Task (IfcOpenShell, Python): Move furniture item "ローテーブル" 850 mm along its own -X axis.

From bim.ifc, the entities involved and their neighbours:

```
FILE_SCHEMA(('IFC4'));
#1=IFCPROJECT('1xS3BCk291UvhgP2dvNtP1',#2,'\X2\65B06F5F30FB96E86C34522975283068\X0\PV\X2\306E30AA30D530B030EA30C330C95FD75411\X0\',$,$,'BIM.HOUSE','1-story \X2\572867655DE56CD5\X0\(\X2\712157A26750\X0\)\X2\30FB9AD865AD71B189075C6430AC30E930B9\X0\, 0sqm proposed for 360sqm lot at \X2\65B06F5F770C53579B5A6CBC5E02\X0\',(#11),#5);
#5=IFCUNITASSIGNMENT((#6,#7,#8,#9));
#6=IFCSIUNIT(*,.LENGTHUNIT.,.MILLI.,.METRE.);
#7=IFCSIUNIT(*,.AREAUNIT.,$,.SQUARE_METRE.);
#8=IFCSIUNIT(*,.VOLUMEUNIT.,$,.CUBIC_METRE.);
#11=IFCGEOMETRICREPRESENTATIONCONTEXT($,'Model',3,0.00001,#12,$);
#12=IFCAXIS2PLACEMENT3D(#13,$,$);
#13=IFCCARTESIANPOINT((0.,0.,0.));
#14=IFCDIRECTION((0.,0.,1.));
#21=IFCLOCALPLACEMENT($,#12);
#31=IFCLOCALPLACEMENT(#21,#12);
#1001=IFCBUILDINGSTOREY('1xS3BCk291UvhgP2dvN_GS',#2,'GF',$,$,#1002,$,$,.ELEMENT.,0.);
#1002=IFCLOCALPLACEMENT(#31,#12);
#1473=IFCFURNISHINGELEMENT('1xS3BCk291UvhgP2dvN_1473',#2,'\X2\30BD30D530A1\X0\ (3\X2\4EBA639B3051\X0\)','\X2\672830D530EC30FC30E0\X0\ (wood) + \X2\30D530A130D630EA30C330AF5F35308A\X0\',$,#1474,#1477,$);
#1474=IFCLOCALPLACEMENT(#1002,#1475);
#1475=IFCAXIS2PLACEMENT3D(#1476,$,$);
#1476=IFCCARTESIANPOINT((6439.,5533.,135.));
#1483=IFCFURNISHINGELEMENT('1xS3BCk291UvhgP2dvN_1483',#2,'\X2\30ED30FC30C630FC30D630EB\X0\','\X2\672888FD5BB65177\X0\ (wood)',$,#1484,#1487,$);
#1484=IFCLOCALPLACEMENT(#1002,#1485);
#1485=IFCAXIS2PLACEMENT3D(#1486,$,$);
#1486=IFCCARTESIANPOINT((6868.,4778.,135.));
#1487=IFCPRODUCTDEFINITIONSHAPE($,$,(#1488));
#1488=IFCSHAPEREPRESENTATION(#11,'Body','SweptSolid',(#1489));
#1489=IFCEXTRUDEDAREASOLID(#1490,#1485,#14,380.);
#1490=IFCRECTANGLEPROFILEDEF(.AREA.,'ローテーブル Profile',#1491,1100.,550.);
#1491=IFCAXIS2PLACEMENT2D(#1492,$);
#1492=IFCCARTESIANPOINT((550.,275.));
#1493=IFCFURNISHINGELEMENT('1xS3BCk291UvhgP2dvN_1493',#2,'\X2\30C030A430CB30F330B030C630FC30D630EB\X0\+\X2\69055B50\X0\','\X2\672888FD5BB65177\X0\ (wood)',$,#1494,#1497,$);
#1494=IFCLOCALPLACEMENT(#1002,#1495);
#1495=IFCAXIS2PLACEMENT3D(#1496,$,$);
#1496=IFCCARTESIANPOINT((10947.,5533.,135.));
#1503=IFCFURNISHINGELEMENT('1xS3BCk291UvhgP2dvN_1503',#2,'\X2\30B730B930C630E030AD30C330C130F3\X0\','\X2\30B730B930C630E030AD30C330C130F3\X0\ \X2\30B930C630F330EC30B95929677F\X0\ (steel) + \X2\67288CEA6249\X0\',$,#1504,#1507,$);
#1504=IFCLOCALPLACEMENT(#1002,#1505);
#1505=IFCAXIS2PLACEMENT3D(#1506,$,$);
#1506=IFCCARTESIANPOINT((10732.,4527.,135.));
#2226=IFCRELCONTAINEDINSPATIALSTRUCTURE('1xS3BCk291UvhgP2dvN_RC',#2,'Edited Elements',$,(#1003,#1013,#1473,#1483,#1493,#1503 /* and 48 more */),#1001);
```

```python
import ifcopenshell
import ifcopenshell.api.geometry
import ifcopenshell.util.placement
import ifcopenshell.util.unit

model = ifcopenshell.open("bim.ifc")
unit_scale = ifcopenshell.util.unit.calculate_unit_scale(model)

item = model.by_guid("1xS3BCk291UvhgP2dvN_1483")
matrix = ifcopenshell.util.placement.get_local_placement(item.ObjectPlacement)
matrix[:3, 3] -= matrix[:3, 0] * 0.85 / unit_scale
ifcopenshell.api.geometry.edit_object_placement(model, product=item, matrix=matrix, is_si=False)

print(ifcopenshell.util.placement.get_local_placement(item.ObjectPlacement).round(3) + 0.0)

model.write("bim_rev.ifc")
```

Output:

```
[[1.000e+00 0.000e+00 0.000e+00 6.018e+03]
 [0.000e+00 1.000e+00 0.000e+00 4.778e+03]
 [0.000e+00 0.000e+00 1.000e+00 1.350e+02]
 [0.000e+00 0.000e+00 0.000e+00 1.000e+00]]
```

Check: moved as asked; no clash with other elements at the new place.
